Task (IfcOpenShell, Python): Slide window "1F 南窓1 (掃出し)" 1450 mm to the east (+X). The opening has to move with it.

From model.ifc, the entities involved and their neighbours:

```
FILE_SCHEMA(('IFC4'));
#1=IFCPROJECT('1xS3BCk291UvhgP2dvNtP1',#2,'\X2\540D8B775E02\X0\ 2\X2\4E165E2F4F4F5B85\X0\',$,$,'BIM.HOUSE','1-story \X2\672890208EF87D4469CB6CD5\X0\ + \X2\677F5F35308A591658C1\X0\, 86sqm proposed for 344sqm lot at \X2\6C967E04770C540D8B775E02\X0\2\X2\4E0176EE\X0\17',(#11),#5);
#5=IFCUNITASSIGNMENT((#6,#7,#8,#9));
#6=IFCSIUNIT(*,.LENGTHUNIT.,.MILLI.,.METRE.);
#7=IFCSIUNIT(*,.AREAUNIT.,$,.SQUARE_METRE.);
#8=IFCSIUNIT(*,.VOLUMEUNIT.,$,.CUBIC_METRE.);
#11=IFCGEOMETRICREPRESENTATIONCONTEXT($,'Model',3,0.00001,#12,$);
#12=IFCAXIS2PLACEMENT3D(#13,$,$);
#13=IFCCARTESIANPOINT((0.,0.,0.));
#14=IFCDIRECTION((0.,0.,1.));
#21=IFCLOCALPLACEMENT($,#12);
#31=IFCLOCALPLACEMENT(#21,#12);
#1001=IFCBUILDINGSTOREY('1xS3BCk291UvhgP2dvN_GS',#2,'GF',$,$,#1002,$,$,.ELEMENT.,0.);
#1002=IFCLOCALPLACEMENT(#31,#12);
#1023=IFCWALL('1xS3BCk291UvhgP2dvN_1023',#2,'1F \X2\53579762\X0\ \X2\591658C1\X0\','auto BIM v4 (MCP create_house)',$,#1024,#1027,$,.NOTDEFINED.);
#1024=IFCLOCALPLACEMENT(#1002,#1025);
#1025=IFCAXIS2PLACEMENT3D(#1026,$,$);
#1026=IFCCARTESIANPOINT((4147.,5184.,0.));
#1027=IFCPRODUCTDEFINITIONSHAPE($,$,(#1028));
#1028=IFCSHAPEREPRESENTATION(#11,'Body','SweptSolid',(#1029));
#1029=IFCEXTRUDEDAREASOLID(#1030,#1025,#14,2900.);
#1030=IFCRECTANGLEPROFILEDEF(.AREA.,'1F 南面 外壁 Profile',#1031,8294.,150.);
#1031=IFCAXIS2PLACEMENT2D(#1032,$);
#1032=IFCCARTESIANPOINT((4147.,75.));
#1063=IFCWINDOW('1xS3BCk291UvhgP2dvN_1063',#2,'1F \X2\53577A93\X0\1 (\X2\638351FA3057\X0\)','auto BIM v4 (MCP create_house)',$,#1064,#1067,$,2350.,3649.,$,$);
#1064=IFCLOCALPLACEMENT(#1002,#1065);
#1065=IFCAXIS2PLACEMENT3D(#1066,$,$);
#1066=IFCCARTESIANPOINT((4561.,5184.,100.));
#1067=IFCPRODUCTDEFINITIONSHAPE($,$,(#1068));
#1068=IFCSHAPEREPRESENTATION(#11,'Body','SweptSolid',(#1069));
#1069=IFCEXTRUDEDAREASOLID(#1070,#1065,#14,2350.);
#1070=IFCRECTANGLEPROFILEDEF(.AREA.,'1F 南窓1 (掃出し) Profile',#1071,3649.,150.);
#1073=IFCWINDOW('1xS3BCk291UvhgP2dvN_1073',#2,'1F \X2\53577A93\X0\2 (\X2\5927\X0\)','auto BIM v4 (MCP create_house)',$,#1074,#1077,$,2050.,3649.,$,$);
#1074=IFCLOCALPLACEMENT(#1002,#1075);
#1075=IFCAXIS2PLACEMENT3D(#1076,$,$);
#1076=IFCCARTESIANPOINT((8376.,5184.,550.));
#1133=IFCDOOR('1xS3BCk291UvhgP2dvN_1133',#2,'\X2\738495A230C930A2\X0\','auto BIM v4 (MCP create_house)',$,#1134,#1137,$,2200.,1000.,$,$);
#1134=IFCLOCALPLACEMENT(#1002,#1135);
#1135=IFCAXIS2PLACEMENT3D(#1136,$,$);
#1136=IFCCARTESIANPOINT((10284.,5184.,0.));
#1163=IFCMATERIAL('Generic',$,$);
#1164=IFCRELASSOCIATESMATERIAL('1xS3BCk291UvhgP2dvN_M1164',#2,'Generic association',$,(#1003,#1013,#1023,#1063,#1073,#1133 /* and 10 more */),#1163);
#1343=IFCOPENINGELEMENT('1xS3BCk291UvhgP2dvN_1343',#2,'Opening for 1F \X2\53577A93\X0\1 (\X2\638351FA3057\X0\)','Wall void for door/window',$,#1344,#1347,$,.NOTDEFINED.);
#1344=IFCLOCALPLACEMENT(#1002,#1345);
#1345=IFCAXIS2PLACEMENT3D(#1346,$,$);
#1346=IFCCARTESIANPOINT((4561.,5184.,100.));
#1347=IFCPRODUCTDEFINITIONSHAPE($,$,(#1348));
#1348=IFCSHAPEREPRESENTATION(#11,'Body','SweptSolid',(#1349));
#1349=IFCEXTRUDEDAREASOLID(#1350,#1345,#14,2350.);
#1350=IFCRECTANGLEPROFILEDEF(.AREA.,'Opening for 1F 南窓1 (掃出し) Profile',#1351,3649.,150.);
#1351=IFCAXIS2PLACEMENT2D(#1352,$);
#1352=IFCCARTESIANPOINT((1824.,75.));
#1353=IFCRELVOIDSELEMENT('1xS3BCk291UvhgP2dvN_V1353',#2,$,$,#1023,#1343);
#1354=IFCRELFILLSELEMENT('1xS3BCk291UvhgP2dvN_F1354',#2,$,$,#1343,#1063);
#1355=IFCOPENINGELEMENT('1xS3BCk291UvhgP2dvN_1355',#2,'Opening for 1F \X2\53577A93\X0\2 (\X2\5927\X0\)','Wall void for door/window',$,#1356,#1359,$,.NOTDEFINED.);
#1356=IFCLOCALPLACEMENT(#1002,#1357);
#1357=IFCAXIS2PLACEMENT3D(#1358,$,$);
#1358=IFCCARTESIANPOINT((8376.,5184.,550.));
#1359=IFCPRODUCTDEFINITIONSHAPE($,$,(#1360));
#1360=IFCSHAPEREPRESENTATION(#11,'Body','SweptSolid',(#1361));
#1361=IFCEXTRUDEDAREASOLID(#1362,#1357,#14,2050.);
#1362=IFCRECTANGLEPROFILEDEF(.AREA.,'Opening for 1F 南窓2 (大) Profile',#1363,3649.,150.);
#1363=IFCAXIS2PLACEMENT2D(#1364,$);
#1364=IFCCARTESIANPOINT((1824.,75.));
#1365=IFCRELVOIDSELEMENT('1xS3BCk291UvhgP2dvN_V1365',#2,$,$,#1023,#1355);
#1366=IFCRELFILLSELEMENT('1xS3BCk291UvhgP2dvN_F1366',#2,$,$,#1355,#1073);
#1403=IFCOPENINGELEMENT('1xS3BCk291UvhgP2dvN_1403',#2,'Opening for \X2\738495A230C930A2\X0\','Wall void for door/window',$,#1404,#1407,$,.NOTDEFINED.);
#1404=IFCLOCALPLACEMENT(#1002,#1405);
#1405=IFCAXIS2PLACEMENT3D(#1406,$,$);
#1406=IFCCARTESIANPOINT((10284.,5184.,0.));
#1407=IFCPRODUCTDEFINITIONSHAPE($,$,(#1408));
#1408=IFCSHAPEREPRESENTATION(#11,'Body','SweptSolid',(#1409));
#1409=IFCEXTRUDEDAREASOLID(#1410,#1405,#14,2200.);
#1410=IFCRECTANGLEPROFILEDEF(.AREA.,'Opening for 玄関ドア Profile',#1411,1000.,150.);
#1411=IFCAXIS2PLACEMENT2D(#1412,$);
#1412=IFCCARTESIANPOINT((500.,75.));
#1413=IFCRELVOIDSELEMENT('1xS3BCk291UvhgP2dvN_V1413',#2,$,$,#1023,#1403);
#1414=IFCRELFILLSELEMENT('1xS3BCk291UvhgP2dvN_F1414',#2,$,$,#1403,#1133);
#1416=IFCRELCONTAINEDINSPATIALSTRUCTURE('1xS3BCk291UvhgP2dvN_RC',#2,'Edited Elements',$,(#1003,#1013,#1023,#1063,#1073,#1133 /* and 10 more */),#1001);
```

```python
import ifcopenshell
import ifcopenshell.api.geometry
import ifcopenshell.util.placement
import ifcopenshell.util.unit

model = ifcopenshell.open("model.ifc")
unit_scale = ifcopenshell.util.unit.calculate_unit_scale(model)

window = model.by_guid("1xS3BCk291UvhgP2dvN_1063")
opening = window.FillsVoids[0].RelatingOpeningElement
wall = opening.VoidsElements[0].RelatingBuildingElement

wall_matrix = ifcopenshell.util.placement.get_local_placement(wall.ObjectPlacement)
shift = wall_matrix[:3, 0] * 1.45 / unit_scale
before = ifcopenshell.util.placement.get_local_placement(window.ObjectPlacement)[:3, 3].copy()

# The window is not placed relative to its opening, so move both.
for product in (opening, window):
    matrix = ifcopenshell.util.placement.get_local_placement(product.ObjectPlacement)
    matrix[:3, 3] += shift
    ifcopenshell.api.geometry.edit_object_placement(model, product=product, matrix=matrix, is_si=False)

after = ifcopenshell.util.placement.get_local_placement(window.ObjectPlacement)[:3, 3]
print("window moved by", (after - before).round(3) + 0.0)

model.write("model_rev.ifc")
```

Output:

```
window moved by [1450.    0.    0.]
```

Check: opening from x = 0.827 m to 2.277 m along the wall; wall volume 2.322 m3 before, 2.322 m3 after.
